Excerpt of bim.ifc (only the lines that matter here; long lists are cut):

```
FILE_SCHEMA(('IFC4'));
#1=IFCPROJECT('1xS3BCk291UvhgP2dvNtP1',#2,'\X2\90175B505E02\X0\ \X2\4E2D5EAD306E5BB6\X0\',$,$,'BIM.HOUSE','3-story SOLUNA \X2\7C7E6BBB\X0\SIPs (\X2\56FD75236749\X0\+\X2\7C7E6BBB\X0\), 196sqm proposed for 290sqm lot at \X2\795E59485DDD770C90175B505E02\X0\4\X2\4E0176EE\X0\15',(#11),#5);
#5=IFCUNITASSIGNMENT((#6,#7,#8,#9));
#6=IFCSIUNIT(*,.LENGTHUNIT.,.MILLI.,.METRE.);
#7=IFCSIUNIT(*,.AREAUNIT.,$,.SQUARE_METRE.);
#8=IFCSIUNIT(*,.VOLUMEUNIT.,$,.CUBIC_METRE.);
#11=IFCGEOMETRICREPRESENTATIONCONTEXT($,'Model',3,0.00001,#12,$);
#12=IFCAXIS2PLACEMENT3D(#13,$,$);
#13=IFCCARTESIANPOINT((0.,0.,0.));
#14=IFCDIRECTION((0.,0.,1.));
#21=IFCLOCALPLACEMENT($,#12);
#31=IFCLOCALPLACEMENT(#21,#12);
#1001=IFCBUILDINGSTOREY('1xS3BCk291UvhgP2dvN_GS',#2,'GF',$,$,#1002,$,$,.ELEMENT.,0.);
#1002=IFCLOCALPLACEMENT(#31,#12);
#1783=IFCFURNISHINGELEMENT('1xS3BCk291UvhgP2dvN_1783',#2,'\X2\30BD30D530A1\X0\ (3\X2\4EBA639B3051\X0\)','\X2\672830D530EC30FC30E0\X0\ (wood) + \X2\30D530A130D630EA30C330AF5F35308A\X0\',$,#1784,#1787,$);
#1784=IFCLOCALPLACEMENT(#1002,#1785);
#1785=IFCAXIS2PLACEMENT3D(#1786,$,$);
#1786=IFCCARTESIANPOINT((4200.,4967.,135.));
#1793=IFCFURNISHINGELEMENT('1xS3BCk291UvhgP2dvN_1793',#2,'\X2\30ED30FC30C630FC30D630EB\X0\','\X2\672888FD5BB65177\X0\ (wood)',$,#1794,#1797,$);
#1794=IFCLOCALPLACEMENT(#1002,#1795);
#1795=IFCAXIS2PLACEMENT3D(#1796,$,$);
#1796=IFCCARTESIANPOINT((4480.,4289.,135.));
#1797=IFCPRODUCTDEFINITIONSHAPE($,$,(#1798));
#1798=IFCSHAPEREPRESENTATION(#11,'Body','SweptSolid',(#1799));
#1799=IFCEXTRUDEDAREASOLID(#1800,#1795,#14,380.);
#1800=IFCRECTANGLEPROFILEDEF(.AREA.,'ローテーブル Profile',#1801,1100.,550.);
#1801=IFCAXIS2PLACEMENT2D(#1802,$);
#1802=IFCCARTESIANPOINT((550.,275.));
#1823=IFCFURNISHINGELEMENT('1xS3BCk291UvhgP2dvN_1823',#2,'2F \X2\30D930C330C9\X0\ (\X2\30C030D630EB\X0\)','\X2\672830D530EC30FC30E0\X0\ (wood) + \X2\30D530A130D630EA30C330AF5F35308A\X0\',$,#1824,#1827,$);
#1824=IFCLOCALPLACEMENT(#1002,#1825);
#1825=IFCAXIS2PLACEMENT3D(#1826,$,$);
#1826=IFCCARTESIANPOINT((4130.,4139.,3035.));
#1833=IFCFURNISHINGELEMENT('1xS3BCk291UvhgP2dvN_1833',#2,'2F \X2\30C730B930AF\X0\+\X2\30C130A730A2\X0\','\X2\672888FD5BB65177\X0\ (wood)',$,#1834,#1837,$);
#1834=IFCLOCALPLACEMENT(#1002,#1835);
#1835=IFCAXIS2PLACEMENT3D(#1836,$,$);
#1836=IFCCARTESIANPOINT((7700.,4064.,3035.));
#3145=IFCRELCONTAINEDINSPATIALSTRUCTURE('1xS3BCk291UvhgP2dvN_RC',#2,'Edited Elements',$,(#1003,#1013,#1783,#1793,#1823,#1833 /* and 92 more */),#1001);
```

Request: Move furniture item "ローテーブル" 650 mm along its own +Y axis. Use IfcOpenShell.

```python
import ifcopenshell
import ifcopenshell.api.geometry
import ifcopenshell.util.placement
import ifcopenshell.util.unit

model = ifcopenshell.open("bim.ifc")
unit_scale = ifcopenshell.util.unit.calculate_unit_scale(model)

item = model.by_guid("1xS3BCk291UvhgP2dvN_1793")
matrix = ifcopenshell.util.placement.get_local_placement(item.ObjectPlacement)
matrix[:3, 3] += matrix[:3, 1] * 0.65 / unit_scale
ifcopenshell.api.geometry.edit_object_placement(model, product=item, matrix=matrix, is_si=False)

print(ifcopenshell.util.placement.get_local_placement(item.ObjectPlacement).round(3) + 0.0)

model.write("bim_rev.ifc")
```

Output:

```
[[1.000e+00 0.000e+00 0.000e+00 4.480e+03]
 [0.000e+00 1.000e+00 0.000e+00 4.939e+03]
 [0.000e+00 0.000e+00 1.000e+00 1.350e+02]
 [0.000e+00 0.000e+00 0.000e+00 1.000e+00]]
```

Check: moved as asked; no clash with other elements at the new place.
